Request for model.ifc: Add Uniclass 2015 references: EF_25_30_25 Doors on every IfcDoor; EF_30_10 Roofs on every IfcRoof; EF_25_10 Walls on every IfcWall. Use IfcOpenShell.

First a look at what the model holds.

```python
import ifcopenshell

model = ifcopenshell.open("model.ifc")
print(model.schema)
print("classifications:", [c.Name for c in model.by_type("IfcClassification")])
for ifc_class in ("IfcDoor", "IfcRoof", "IfcStair", "IfcWall", "IfcWindow"):
    print(ifc_class, len(model.by_type(ifc_class)))
```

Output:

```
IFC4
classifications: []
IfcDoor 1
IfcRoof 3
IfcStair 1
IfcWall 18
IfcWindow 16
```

```python
import ifcopenshell
import ifcopenshell.api.classification

model = ifcopenshell.open("model.ifc")

system = ifcopenshell.api.classification.add_classification(model, classification="Uniclass 2015")

codes = {
    "IfcDoor": ("EF_25_30_25", "Doors"),
    "IfcRoof": ("EF_30_10", "Roofs"),
    "IfcWall": ("EF_25_10", "Walls"),
}
for ifc_class, (code, name) in codes.items():
    products = model.by_type(ifc_class)
    ifcopenshell.api.classification.add_reference(
        model, products=products, classification=system, identification=code, name=name
    )
    print(code, len(products))

model.write("model_v2.ifc")
```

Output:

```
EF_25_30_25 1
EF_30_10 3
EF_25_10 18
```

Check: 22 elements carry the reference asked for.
